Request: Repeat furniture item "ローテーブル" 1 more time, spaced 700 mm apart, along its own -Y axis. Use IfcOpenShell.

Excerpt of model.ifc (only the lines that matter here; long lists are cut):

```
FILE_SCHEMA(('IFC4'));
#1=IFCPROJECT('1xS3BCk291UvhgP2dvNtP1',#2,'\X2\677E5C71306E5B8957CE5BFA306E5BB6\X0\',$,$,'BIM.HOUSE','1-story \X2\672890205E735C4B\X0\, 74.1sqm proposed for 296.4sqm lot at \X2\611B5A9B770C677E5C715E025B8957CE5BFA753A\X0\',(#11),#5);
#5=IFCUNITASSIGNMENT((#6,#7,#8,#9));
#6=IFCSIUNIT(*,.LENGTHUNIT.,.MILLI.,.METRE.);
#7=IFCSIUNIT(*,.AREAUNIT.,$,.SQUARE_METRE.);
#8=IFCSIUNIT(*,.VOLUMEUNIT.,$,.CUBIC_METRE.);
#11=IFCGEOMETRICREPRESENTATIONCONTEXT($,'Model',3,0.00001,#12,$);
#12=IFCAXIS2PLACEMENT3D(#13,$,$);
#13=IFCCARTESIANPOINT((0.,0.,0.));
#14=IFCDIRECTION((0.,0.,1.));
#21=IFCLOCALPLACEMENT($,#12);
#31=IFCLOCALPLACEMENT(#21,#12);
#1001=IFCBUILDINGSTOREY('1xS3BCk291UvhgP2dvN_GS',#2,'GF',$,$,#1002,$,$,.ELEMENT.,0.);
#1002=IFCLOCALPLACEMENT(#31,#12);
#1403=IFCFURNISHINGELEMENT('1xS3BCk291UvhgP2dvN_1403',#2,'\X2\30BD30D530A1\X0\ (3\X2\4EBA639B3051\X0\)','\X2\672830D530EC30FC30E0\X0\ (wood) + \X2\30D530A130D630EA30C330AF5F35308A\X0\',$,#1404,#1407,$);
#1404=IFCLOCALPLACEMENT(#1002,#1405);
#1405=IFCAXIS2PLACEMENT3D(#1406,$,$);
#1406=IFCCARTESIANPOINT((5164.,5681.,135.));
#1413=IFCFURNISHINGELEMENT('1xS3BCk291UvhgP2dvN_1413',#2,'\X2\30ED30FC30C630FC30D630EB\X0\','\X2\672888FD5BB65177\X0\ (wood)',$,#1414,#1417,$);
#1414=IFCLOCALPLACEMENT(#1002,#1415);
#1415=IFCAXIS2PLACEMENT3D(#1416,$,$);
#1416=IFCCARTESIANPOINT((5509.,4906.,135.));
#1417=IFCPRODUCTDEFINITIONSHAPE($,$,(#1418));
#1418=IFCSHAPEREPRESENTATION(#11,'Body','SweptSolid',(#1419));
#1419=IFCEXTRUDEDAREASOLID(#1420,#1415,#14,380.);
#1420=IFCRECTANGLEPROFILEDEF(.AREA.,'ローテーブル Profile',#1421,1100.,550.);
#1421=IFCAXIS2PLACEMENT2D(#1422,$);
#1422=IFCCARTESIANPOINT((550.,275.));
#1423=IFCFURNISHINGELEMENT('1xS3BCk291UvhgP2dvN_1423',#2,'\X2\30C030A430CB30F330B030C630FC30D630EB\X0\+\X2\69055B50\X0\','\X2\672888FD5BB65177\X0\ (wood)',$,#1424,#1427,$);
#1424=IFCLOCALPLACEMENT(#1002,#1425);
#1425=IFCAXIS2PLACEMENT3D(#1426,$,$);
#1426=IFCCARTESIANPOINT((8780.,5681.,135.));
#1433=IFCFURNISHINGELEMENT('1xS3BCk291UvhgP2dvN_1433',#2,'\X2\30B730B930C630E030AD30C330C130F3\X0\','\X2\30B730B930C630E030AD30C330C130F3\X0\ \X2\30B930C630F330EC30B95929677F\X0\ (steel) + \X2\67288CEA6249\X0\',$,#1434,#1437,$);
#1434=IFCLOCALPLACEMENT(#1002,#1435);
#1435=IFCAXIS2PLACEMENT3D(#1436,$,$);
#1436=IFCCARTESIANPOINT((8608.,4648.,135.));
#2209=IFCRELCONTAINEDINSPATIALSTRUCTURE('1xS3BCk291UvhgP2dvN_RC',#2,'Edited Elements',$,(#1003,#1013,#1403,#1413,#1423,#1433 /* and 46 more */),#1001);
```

```python
import ifcopenshell
import ifcopenshell.api.geometry
import ifcopenshell.api.root
import ifcopenshell.util.element
import ifcopenshell.util.placement

model = ifcopenshell.open("model.ifc")


def reuse_history(source, copy):
    """copy_class also copies each property set's owner history, people and application; keep the originals."""
    for rel in copy.IsDefinedBy:
        if rel.is_a("IfcRelDefinesByProperties") and (history := rel.RelatingPropertyDefinition.OwnerHistory):
            rel.RelatingPropertyDefinition.OwnerHistory = source.OwnerHistory
            ifcopenshell.util.element.remove_deep2(model, history)


source = model.by_guid("1xS3BCk291UvhgP2dvN_1413")
base = ifcopenshell.util.placement.get_local_placement(source.ObjectPlacement)
step = -base[:3, 1] * 700.0

for i in range(1, 2):
    copy = ifcopenshell.api.root.copy_class(model, product=source)
    copy.Representation = ifcopenshell.util.element.copy_deep(
        model, source.Representation, exclude=["IfcGeometricRepresentationContext", "IfcRepresentationMap"]
    )
    reuse_history(source, copy)
    matrix = base.copy()
    matrix[:3, 3] += i * step
    print("added at", matrix[:3, 3].round(3) + 0.0)
    ifcopenshell.api.geometry.edit_object_placement(model, product=copy, matrix=matrix, is_si=False)

model.write("model_rev.ifc")
```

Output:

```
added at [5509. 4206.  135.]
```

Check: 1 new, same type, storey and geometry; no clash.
